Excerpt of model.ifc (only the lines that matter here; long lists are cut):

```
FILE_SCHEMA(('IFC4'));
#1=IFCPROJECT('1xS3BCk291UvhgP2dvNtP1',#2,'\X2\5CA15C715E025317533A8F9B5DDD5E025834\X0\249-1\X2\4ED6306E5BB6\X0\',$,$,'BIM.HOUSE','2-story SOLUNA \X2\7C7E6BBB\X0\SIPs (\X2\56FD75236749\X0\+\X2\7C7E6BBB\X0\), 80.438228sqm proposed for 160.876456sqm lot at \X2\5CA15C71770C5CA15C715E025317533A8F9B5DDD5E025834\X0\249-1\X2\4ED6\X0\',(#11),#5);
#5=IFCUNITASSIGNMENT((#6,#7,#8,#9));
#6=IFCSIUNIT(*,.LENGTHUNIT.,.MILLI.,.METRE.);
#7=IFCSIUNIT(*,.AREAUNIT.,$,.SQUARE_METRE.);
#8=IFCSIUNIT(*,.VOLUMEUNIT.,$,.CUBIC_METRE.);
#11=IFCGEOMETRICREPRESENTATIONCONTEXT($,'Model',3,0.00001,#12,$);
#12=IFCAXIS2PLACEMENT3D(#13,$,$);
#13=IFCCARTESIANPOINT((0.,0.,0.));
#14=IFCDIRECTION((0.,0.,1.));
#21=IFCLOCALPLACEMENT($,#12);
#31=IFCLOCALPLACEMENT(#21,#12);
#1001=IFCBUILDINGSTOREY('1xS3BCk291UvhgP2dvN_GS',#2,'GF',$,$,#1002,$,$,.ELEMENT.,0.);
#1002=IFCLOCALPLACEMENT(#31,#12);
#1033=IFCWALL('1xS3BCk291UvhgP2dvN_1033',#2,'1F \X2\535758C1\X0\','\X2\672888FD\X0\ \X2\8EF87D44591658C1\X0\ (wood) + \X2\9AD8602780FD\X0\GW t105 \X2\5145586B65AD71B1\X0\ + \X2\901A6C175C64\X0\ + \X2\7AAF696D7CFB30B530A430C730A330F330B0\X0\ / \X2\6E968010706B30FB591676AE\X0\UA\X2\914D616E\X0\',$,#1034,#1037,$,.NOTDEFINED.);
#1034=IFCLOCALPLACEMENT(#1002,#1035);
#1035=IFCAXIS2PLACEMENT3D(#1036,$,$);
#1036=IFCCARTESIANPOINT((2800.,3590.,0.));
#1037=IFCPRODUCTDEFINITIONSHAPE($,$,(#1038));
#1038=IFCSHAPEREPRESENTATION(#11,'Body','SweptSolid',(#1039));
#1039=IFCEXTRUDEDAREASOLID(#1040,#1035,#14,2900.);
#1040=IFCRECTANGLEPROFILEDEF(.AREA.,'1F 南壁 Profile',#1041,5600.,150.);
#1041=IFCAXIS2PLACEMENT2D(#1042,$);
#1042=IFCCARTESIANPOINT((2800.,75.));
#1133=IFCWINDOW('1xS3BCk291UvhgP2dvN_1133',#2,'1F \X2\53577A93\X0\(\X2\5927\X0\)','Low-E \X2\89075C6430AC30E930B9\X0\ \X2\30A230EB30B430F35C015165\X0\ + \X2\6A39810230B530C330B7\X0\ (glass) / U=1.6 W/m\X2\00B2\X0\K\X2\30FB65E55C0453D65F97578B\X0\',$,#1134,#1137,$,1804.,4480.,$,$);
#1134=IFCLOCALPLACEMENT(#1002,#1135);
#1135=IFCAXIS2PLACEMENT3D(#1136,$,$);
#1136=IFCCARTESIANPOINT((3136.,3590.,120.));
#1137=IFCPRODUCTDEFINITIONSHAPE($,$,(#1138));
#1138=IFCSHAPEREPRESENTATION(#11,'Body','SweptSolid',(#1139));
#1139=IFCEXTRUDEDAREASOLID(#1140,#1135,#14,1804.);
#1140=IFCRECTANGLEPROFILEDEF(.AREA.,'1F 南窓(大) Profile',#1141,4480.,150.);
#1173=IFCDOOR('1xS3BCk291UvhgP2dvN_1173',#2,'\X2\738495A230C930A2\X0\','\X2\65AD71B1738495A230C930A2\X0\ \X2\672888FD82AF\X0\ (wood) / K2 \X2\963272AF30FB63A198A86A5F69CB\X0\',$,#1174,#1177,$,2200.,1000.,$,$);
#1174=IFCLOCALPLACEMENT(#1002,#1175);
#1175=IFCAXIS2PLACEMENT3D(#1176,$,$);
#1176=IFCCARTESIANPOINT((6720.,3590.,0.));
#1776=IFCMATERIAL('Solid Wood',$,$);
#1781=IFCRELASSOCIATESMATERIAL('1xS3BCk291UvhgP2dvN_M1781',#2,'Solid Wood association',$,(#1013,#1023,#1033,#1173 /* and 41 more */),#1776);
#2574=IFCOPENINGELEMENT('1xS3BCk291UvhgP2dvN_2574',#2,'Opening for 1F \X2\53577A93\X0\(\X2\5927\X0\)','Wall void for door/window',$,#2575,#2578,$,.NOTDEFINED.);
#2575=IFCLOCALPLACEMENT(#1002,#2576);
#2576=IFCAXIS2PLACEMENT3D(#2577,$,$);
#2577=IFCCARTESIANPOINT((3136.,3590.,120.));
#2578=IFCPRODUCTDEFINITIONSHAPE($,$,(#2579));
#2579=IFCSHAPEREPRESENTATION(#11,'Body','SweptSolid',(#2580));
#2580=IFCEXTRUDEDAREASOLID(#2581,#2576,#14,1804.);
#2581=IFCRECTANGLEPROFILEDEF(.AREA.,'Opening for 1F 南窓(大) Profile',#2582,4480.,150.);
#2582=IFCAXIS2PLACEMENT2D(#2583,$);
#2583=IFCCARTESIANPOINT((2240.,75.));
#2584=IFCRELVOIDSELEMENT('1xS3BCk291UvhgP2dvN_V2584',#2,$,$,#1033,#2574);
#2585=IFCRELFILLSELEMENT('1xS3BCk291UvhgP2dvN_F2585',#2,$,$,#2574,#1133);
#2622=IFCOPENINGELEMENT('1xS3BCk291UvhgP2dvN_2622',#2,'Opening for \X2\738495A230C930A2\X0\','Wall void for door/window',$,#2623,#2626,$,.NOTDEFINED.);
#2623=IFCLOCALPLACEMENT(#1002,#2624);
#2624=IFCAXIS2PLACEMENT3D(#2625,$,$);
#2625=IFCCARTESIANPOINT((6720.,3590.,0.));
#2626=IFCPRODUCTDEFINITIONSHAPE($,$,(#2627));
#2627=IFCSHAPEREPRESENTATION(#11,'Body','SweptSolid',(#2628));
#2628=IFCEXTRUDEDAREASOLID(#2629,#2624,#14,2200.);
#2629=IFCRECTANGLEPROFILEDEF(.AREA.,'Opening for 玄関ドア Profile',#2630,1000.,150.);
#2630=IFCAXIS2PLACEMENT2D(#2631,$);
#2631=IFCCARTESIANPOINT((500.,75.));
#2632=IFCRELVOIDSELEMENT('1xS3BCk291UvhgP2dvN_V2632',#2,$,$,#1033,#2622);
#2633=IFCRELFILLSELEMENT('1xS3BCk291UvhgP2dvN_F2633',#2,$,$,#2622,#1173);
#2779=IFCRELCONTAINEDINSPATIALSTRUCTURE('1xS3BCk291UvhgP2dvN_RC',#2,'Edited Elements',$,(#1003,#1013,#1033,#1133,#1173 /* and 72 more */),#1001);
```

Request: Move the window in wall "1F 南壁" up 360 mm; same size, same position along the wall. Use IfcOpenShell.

```python
import numpy as np
import ifcopenshell
import ifcopenshell.api.geometry
import ifcopenshell.util.placement
import ifcopenshell.util.unit

model = ifcopenshell.open("model.ifc")
unit_scale = ifcopenshell.util.unit.calculate_unit_scale(model)

window = model.by_guid("1xS3BCk291UvhgP2dvN_1133")
opening = window.FillsVoids[0].RelatingOpeningElement
dz = 0.36 / unit_scale

shift = np.array([0.0, 0.0, dz])
# The window is not placed relative to its opening, so move both.
for product in (opening, window):
    matrix = ifcopenshell.util.placement.get_local_placement(product.ObjectPlacement)
    matrix[:3, 3] += shift
    ifcopenshell.api.geometry.edit_object_placement(model, product=product, matrix=matrix, is_si=False)

print(f"moved by {dz * unit_scale:+.3f} m")

model.write("model_edited.ifc")
```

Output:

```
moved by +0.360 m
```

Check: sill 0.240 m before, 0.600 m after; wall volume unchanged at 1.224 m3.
